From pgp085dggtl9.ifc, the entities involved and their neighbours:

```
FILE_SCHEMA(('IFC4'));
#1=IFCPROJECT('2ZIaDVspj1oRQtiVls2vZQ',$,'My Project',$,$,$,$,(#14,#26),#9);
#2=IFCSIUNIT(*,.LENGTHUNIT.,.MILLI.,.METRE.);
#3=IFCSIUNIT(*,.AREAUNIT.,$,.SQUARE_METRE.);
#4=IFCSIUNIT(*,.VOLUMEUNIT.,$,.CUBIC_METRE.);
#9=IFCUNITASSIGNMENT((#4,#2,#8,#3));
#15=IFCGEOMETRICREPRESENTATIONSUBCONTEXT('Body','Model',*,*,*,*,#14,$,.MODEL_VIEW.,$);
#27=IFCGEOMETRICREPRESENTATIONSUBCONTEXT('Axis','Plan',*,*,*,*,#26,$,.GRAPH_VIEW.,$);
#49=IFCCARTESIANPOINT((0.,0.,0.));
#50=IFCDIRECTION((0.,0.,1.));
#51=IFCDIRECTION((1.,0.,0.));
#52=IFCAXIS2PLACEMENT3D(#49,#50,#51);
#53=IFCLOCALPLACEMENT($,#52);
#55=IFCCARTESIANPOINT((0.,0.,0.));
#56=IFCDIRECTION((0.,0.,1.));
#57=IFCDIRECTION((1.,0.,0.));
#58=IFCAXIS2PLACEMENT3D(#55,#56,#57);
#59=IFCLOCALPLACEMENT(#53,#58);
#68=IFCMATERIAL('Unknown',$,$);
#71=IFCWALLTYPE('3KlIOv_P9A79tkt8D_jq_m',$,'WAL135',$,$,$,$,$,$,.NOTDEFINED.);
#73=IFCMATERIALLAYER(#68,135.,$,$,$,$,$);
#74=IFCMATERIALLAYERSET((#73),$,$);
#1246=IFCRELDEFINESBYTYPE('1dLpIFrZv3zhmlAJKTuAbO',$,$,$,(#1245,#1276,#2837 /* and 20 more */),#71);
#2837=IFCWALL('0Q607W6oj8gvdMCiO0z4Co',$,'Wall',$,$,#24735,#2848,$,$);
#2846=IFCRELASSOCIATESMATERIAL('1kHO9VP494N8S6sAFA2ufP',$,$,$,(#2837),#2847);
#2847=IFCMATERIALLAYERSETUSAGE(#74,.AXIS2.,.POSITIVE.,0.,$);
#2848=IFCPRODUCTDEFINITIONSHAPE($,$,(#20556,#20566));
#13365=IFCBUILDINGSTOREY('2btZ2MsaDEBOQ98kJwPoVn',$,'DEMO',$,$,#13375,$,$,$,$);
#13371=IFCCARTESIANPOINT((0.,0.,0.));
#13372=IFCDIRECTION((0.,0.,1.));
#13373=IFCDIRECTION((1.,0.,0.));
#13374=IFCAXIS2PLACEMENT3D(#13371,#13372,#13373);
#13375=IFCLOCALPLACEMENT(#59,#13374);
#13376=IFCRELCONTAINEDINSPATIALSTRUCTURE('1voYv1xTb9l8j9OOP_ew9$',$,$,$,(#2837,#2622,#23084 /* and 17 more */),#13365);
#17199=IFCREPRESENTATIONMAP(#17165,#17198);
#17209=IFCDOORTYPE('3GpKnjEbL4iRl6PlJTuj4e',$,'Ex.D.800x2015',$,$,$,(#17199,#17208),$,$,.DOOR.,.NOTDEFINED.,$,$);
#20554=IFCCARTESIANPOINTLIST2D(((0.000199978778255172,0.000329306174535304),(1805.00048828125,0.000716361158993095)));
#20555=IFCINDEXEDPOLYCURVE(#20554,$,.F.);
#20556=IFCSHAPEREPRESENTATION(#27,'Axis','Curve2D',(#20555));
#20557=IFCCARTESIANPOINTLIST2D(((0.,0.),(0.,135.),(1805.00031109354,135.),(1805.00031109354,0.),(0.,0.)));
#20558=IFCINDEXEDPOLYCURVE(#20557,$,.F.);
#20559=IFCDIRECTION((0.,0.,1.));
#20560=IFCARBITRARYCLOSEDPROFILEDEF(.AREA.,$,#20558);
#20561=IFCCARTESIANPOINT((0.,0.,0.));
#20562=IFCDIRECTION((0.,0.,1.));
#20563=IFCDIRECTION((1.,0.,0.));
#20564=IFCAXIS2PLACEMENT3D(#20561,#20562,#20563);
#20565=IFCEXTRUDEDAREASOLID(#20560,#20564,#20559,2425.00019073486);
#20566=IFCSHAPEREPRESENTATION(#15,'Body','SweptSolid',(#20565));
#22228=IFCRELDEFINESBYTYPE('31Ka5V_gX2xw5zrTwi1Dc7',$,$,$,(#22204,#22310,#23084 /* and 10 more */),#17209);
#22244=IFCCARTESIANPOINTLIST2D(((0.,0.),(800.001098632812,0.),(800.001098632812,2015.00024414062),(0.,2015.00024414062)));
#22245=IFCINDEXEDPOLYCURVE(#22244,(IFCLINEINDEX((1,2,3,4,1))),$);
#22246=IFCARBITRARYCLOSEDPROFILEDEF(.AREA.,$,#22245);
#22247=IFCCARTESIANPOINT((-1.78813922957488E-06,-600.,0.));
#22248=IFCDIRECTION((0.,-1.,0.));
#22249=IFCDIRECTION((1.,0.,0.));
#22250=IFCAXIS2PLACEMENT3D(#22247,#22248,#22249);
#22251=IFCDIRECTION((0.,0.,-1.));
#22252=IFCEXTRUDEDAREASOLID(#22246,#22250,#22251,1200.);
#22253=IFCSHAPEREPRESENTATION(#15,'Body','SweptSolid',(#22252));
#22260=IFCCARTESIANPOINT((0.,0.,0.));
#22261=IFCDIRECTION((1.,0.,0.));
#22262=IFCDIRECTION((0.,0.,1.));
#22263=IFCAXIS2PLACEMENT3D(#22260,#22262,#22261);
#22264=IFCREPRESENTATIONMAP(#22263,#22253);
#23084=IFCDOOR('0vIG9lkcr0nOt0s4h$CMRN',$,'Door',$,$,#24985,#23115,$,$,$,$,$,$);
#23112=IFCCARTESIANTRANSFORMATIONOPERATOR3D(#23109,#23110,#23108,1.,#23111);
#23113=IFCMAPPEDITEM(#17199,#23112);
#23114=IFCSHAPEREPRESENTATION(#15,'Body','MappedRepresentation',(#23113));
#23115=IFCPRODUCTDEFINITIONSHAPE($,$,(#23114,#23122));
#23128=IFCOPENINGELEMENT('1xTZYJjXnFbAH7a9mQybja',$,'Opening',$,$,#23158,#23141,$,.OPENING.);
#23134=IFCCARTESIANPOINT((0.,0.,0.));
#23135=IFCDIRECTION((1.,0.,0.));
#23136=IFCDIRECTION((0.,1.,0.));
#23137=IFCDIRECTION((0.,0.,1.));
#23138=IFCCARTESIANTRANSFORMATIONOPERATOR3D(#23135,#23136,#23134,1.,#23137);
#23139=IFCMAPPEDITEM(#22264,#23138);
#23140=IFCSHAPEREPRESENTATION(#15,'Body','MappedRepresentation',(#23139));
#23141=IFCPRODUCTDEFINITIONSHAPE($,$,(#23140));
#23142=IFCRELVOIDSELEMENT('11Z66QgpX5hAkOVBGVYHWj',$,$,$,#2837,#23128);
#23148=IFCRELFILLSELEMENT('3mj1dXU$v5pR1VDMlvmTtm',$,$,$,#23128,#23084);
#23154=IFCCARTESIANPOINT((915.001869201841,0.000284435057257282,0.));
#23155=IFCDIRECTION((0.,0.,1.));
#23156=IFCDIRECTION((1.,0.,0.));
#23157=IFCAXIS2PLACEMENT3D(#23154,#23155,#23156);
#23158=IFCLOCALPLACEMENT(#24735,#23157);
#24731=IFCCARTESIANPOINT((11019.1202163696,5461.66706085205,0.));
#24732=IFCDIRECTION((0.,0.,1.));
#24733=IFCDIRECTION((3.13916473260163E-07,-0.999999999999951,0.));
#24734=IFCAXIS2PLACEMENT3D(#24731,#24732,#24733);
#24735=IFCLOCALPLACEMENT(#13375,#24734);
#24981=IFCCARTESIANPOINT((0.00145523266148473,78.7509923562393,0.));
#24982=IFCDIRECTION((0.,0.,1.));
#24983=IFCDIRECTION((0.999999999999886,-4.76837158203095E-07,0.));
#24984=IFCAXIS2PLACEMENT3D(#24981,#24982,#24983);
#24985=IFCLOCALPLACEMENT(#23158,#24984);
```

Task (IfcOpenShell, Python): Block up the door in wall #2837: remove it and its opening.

```python
import ifcopenshell
import ifcopenshell.api.feature
import ifcopenshell.api.root
import ifcopenshell.geom
import ifcopenshell.util.shape

model = ifcopenshell.open("pgp085dggtl9.ifc")
settings = ifcopenshell.geom.settings()


def volume(element):
    """Net volume in cubic metres, openings subtracted."""
    shape = ifcopenshell.geom.create_shape(settings, element)
    return ifcopenshell.util.shape.get_volume(shape.geometry)


door = model.by_guid("0vIG9lkcr0nOt0s4h$CMRN")
opening = door.FillsVoids[0].RelatingOpeningElement
wall = opening.VoidsElements[0].RelatingBuildingElement
before = volume(wall)

ifcopenshell.api.root.remove_product(model, product=door)
ifcopenshell.api.feature.remove_feature(model, feature=opening)

after = volume(wall)

print(f"wall volume {before:.3f} -> {after:.3f} m3")

model.write("pgp085dggtl9-out.ifc")
```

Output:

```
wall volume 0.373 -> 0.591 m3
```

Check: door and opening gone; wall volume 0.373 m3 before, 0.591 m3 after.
